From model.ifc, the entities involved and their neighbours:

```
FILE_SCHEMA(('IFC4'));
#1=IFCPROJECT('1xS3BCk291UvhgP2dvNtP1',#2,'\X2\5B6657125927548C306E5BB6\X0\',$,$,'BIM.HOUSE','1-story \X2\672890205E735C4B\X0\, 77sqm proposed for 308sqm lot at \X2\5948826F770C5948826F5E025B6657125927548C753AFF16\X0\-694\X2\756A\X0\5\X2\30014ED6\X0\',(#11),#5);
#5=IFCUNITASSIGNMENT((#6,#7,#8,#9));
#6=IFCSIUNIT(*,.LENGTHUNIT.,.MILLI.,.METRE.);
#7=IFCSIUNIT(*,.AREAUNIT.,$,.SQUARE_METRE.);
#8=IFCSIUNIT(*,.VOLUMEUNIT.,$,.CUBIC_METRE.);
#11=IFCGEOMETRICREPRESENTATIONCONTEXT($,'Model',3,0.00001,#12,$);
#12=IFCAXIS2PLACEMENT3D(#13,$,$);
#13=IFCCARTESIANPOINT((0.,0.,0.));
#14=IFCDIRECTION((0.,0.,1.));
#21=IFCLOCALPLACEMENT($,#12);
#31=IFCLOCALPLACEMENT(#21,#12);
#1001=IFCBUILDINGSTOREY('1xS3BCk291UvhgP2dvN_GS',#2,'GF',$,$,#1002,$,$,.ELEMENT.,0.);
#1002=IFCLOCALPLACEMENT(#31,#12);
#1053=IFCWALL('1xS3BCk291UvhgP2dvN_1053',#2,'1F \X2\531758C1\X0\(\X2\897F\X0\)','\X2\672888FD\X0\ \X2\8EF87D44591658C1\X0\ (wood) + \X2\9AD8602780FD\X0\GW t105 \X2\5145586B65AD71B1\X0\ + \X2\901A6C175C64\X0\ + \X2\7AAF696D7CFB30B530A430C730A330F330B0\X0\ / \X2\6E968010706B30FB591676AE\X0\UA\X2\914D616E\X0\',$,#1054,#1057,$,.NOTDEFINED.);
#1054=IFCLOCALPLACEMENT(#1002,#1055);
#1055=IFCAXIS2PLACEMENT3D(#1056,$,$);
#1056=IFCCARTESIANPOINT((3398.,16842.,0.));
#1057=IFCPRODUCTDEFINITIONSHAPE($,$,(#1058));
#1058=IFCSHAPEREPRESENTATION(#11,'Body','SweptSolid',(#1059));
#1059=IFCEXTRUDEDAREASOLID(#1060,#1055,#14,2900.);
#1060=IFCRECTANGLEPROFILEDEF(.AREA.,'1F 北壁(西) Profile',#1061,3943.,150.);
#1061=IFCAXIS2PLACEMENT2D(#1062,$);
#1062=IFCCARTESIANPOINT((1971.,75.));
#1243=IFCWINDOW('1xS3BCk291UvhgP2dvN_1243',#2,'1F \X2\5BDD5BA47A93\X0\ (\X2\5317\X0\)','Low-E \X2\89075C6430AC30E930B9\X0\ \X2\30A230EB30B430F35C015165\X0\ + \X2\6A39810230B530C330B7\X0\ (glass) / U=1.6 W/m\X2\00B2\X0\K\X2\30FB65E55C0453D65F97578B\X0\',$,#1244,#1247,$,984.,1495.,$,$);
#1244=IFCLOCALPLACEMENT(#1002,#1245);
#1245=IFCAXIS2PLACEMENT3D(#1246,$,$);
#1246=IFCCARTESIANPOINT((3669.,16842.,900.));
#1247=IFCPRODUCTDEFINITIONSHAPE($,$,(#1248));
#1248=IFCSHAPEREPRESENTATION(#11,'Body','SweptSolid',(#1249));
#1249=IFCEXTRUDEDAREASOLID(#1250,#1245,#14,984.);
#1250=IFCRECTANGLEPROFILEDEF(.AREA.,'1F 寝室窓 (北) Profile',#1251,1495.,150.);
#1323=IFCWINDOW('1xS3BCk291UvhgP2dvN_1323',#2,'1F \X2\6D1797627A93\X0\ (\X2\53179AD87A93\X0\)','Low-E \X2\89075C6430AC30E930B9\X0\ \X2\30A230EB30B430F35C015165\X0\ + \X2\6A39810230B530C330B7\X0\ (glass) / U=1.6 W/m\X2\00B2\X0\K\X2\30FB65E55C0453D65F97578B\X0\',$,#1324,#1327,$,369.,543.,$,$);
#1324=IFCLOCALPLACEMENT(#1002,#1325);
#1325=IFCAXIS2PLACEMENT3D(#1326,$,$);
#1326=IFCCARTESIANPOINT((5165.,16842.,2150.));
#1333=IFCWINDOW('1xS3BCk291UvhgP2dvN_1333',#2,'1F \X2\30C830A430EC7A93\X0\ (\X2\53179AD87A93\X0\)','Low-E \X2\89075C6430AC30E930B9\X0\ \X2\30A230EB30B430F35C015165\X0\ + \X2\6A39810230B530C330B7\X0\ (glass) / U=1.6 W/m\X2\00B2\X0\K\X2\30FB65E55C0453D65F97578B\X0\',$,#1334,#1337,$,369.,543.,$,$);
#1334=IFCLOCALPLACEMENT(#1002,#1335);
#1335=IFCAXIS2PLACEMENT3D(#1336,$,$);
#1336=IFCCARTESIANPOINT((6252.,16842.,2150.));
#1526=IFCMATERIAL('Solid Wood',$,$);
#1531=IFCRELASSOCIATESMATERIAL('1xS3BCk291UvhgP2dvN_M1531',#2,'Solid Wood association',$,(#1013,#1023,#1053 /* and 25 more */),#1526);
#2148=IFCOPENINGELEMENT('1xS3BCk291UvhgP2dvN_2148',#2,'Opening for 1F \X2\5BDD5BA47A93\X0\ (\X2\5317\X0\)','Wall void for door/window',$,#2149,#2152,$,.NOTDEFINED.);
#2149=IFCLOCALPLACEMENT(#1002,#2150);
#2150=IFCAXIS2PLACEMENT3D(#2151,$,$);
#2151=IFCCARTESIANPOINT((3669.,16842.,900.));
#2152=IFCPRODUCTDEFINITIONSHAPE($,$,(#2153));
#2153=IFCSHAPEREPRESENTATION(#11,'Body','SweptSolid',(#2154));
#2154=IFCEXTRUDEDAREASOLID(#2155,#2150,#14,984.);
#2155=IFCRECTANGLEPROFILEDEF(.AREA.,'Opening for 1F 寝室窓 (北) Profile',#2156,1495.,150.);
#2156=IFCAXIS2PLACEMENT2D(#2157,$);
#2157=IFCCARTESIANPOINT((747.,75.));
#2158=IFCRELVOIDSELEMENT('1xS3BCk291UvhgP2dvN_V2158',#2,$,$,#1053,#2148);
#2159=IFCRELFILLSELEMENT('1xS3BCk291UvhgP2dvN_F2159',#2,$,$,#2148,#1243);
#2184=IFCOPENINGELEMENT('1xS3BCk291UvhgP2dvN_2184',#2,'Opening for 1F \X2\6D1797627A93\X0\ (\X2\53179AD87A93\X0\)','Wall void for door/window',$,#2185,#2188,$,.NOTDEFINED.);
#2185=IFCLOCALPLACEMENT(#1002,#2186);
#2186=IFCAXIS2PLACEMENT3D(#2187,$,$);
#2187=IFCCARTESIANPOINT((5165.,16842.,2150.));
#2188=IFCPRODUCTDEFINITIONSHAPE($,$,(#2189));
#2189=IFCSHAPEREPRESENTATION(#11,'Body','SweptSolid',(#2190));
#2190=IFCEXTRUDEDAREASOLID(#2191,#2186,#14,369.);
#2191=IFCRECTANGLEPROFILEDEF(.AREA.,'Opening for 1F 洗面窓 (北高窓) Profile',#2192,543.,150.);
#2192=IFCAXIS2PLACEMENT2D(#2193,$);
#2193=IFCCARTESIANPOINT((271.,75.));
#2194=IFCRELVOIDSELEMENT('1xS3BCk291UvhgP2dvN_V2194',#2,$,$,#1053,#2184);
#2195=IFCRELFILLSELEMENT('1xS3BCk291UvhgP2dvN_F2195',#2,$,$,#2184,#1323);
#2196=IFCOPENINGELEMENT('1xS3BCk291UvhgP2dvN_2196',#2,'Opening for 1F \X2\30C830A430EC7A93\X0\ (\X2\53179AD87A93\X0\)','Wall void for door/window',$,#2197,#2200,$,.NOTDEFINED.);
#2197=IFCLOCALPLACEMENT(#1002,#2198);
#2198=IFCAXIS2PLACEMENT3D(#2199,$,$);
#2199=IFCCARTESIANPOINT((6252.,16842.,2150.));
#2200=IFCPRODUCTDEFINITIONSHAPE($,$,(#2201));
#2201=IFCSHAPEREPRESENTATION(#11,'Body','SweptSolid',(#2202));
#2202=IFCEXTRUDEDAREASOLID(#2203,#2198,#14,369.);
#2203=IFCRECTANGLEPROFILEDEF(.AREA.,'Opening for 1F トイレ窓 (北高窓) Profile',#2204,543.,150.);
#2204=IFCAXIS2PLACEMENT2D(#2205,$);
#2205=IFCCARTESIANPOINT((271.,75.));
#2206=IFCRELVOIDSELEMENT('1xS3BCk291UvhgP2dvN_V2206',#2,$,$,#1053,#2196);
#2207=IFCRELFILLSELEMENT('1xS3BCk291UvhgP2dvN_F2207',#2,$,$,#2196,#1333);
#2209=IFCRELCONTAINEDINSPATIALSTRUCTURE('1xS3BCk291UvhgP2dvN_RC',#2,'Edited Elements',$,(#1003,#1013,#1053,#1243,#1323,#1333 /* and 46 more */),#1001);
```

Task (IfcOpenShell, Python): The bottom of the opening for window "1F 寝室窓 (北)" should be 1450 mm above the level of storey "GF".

```python
import numpy as np
import ifcopenshell
import ifcopenshell.api.geometry
import ifcopenshell.geom
import ifcopenshell.util.element
import ifcopenshell.util.placement
import ifcopenshell.util.shape
import ifcopenshell.util.unit

model = ifcopenshell.open("model.ifc")
unit_scale = ifcopenshell.util.unit.calculate_unit_scale(model)

window = model.by_id(1243)
opening = window.FillsVoids[0].RelatingOpeningElement
storey = ifcopenshell.util.element.get_container(window, ifc_class="IfcBuildingStorey")
level = ifcopenshell.util.placement.get_local_placement(storey.ObjectPlacement)[2, 3]

# The opening's origin need not be at the sill, so measure its lowest point.
shape = ifcopenshell.geom.create_shape(ifcopenshell.geom.settings(), opening)
bottom = ifcopenshell.util.shape.get_shape_bottom_elevation(shape, shape.geometry) / unit_scale
dz = level + 1450.0 - bottom

shift = np.array([0.0, 0.0, dz])
# The window is not placed relative to its opening, so move both.
for product in (opening, window):
    matrix = ifcopenshell.util.placement.get_local_placement(product.ObjectPlacement)
    matrix[:3, 3] += shift
    ifcopenshell.api.geometry.edit_object_placement(model, product=product, matrix=matrix, is_si=False)

print(f"moved by {dz * unit_scale:+.3f} m")

model.write("model_v2.ifc")
```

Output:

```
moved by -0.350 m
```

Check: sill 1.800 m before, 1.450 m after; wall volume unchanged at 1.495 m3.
